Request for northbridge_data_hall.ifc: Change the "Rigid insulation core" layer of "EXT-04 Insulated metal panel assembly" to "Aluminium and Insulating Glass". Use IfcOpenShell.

First a look at what the model holds.

```python
import ifcopenshell
import ifcopenshell.util.element

model = ifcopenshell.open("northbridge_data_hall.ifc")
print(model.schema)
for layer_set in model.by_type("IfcMaterialLayerSet"):
    if layer_set.LayerSetName == "EXT-04 Insulated metal panel assembly":
        for layer in layer_set.MaterialLayers:
            print(layer.id(), layer.Material and layer.Material.Name, layer.LayerThickness, sep=" | ")
        print(len(ifcopenshell.util.element.get_elements_by_material(model, layer_set)), "elements and types use it")
print(sorted(m.Name for m in model.by_type("IfcMaterial") if m.Name)[:60])
```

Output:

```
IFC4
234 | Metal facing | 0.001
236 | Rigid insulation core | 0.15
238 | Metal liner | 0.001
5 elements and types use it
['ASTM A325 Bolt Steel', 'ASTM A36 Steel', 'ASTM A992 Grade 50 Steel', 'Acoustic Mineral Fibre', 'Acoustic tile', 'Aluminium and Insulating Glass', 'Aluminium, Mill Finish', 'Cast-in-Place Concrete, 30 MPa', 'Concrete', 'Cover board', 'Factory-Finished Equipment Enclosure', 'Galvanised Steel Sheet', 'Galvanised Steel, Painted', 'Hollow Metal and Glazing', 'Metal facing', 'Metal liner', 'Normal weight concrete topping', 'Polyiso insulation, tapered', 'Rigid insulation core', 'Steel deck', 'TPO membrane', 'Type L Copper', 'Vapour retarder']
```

```python
import ifcopenshell
import ifcopenshell.api.material

model = ifcopenshell.open("northbridge_data_hall.ifc")

layer_set = next(s for s in model.by_type("IfcMaterialLayerSet") if s.LayerSetName == "EXT-04 Insulated metal panel assembly")
layer = next(l for l in layer_set.MaterialLayers if l.Material and l.Material.Name == "Rigid insulation core")
material = next(m for m in model.by_type("IfcMaterial") if m.Name == "Aluminium and Insulating Glass")

# Point this one layer at the other material; renaming the old one would change it everywhere.
ifcopenshell.api.material.edit_layer(model, layer=layer, attributes={"Name": material.Name}, material=material)

print([l.Material.Name if l.Material else None for l in layer_set.MaterialLayers])

model.write("northbridge_data_hall-out.ifc")
```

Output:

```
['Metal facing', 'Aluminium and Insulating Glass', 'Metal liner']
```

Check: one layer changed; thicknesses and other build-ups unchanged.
